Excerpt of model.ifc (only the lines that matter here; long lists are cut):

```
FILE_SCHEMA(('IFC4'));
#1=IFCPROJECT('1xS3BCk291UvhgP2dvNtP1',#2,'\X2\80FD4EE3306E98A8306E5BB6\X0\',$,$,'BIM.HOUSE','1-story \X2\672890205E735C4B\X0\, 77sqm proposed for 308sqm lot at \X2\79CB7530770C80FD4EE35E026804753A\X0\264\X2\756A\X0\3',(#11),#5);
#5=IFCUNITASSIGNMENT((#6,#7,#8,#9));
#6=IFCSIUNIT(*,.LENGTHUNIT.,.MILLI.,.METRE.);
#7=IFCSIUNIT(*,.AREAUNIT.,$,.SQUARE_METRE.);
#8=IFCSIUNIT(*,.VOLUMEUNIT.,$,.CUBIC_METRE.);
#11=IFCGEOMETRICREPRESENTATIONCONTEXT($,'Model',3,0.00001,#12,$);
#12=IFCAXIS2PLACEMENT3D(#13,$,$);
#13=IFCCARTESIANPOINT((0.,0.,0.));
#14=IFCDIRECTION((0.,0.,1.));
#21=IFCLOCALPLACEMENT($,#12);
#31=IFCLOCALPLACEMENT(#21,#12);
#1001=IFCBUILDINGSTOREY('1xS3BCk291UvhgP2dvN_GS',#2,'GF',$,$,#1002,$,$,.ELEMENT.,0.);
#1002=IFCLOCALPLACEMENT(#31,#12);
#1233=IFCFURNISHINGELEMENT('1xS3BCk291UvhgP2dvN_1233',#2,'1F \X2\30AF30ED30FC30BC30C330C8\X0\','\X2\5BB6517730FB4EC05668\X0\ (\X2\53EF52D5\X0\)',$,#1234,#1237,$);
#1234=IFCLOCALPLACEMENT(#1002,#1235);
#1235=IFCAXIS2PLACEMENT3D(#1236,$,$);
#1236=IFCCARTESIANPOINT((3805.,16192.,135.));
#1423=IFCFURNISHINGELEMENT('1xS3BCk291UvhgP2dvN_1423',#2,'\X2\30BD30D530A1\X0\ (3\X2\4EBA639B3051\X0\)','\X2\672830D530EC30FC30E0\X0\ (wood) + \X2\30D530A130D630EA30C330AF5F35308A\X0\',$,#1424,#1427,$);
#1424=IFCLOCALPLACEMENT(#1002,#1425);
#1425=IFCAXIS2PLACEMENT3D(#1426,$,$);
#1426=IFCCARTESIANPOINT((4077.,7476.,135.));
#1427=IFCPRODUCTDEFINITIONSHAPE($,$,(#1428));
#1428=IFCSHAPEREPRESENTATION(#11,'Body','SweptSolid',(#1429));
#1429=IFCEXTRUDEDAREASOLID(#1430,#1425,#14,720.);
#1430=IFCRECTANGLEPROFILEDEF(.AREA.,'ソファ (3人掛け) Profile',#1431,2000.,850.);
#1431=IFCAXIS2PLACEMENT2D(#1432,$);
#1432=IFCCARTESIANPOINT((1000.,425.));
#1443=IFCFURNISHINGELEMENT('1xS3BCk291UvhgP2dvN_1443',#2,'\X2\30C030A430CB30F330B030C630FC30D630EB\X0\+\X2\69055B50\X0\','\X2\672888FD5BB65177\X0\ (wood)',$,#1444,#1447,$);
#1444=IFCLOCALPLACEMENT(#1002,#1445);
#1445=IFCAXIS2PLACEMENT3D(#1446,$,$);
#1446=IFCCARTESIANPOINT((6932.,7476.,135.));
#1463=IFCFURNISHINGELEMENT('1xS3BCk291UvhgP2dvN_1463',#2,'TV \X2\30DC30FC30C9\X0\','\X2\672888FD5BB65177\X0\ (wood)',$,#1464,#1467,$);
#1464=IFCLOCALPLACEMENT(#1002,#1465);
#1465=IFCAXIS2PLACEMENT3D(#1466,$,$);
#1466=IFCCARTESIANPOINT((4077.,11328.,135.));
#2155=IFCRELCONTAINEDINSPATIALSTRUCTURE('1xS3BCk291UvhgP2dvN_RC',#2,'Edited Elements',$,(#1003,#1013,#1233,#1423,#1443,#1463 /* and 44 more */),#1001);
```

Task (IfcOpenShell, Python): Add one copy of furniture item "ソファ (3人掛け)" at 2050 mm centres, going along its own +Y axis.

```python
import ifcopenshell
import ifcopenshell.api.geometry
import ifcopenshell.api.root
import ifcopenshell.util.element
import ifcopenshell.util.placement

model = ifcopenshell.open("model.ifc")


def reuse_history(source, copy):
    """copy_class also copies each property set's owner history, people and application; keep the originals."""
    for rel in copy.IsDefinedBy:
        if rel.is_a("IfcRelDefinesByProperties") and (history := rel.RelatingPropertyDefinition.OwnerHistory):
            rel.RelatingPropertyDefinition.OwnerHistory = source.OwnerHistory
            ifcopenshell.util.element.remove_deep2(model, history)


source = model.by_guid("1xS3BCk291UvhgP2dvN_1423")
base = ifcopenshell.util.placement.get_local_placement(source.ObjectPlacement)
step = base[:3, 1] * 2050.0

for i in range(1, 2):
    copy = ifcopenshell.api.root.copy_class(model, product=source)
    copy.Representation = ifcopenshell.util.element.copy_deep(
        model, source.Representation, exclude=["IfcGeometricRepresentationContext", "IfcRepresentationMap"]
    )
    reuse_history(source, copy)
    matrix = base.copy()
    matrix[:3, 3] += i * step
    print("added at", matrix[:3, 3].round(3) + 0.0)
    ifcopenshell.api.geometry.edit_object_placement(model, product=copy, matrix=matrix, is_si=False)

model.write("model_updated.ifc")
```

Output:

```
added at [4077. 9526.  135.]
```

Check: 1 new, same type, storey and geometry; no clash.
